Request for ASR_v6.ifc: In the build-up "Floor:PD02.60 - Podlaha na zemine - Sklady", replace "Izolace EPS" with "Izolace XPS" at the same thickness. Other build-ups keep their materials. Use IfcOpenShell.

First a look at what the model holds.

```python
import ifcopenshell
import ifcopenshell.util.element

model = ifcopenshell.open("ASR_v6.ifc")
print(model.schema)
for layer_set in model.by_type("IfcMaterialLayerSet"):
    if layer_set.LayerSetName == "Floor:PD02.60 - Podlaha na zemine - Sklady":
        for layer in layer_set.MaterialLayers:
            print(layer.id(), layer.Material and layer.Material.Name, layer.LayerThickness, sep=" | ")
        print(len(ifcopenshell.util.element.get_elements_by_material(model, layer_set)), "elements and types use it")
print(sorted(m.Name for m in model.by_type("IfcMaterial") if m.Name)[:60])
```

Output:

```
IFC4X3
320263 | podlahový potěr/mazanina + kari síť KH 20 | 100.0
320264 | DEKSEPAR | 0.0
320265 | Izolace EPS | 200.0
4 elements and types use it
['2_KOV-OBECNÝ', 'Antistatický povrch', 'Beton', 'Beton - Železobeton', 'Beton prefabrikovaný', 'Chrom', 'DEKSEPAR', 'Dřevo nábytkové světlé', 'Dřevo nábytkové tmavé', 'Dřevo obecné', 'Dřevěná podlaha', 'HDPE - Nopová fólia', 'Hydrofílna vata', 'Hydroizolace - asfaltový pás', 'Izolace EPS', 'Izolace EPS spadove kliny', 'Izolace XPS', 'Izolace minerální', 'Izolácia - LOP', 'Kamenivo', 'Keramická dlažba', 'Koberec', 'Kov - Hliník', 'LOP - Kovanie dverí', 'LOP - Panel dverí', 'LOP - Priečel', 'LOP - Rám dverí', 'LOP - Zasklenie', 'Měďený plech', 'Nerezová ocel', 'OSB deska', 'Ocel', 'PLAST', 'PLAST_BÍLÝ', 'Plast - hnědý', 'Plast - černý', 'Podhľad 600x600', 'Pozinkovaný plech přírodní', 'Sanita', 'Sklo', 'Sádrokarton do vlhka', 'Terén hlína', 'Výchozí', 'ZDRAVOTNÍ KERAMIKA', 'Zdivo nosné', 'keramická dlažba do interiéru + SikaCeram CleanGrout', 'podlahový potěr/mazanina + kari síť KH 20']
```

```python
import ifcopenshell
import ifcopenshell.api.material

model = ifcopenshell.open("ASR_v6.ifc")

layer_set = next(s for s in model.by_type("IfcMaterialLayerSet") if s.LayerSetName == "Floor:PD02.60 - Podlaha na zemine - Sklady")
layer = next(l for l in layer_set.MaterialLayers if l.Material and l.Material.Name == "Izolace EPS")
material = next(m for m in model.by_type("IfcMaterial") if m.Name == "Izolace XPS")

# Point this one layer at the other material; renaming the old one would change it everywhere.
ifcopenshell.api.material.edit_layer(model, layer=layer, attributes={"Name": material.Name}, material=material)

print([l.Material.Name if l.Material else None for l in layer_set.MaterialLayers])

model.write("ASR_v6_v2.ifc")
```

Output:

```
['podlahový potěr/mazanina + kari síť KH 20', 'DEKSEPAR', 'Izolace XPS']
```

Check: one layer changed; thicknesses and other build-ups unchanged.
